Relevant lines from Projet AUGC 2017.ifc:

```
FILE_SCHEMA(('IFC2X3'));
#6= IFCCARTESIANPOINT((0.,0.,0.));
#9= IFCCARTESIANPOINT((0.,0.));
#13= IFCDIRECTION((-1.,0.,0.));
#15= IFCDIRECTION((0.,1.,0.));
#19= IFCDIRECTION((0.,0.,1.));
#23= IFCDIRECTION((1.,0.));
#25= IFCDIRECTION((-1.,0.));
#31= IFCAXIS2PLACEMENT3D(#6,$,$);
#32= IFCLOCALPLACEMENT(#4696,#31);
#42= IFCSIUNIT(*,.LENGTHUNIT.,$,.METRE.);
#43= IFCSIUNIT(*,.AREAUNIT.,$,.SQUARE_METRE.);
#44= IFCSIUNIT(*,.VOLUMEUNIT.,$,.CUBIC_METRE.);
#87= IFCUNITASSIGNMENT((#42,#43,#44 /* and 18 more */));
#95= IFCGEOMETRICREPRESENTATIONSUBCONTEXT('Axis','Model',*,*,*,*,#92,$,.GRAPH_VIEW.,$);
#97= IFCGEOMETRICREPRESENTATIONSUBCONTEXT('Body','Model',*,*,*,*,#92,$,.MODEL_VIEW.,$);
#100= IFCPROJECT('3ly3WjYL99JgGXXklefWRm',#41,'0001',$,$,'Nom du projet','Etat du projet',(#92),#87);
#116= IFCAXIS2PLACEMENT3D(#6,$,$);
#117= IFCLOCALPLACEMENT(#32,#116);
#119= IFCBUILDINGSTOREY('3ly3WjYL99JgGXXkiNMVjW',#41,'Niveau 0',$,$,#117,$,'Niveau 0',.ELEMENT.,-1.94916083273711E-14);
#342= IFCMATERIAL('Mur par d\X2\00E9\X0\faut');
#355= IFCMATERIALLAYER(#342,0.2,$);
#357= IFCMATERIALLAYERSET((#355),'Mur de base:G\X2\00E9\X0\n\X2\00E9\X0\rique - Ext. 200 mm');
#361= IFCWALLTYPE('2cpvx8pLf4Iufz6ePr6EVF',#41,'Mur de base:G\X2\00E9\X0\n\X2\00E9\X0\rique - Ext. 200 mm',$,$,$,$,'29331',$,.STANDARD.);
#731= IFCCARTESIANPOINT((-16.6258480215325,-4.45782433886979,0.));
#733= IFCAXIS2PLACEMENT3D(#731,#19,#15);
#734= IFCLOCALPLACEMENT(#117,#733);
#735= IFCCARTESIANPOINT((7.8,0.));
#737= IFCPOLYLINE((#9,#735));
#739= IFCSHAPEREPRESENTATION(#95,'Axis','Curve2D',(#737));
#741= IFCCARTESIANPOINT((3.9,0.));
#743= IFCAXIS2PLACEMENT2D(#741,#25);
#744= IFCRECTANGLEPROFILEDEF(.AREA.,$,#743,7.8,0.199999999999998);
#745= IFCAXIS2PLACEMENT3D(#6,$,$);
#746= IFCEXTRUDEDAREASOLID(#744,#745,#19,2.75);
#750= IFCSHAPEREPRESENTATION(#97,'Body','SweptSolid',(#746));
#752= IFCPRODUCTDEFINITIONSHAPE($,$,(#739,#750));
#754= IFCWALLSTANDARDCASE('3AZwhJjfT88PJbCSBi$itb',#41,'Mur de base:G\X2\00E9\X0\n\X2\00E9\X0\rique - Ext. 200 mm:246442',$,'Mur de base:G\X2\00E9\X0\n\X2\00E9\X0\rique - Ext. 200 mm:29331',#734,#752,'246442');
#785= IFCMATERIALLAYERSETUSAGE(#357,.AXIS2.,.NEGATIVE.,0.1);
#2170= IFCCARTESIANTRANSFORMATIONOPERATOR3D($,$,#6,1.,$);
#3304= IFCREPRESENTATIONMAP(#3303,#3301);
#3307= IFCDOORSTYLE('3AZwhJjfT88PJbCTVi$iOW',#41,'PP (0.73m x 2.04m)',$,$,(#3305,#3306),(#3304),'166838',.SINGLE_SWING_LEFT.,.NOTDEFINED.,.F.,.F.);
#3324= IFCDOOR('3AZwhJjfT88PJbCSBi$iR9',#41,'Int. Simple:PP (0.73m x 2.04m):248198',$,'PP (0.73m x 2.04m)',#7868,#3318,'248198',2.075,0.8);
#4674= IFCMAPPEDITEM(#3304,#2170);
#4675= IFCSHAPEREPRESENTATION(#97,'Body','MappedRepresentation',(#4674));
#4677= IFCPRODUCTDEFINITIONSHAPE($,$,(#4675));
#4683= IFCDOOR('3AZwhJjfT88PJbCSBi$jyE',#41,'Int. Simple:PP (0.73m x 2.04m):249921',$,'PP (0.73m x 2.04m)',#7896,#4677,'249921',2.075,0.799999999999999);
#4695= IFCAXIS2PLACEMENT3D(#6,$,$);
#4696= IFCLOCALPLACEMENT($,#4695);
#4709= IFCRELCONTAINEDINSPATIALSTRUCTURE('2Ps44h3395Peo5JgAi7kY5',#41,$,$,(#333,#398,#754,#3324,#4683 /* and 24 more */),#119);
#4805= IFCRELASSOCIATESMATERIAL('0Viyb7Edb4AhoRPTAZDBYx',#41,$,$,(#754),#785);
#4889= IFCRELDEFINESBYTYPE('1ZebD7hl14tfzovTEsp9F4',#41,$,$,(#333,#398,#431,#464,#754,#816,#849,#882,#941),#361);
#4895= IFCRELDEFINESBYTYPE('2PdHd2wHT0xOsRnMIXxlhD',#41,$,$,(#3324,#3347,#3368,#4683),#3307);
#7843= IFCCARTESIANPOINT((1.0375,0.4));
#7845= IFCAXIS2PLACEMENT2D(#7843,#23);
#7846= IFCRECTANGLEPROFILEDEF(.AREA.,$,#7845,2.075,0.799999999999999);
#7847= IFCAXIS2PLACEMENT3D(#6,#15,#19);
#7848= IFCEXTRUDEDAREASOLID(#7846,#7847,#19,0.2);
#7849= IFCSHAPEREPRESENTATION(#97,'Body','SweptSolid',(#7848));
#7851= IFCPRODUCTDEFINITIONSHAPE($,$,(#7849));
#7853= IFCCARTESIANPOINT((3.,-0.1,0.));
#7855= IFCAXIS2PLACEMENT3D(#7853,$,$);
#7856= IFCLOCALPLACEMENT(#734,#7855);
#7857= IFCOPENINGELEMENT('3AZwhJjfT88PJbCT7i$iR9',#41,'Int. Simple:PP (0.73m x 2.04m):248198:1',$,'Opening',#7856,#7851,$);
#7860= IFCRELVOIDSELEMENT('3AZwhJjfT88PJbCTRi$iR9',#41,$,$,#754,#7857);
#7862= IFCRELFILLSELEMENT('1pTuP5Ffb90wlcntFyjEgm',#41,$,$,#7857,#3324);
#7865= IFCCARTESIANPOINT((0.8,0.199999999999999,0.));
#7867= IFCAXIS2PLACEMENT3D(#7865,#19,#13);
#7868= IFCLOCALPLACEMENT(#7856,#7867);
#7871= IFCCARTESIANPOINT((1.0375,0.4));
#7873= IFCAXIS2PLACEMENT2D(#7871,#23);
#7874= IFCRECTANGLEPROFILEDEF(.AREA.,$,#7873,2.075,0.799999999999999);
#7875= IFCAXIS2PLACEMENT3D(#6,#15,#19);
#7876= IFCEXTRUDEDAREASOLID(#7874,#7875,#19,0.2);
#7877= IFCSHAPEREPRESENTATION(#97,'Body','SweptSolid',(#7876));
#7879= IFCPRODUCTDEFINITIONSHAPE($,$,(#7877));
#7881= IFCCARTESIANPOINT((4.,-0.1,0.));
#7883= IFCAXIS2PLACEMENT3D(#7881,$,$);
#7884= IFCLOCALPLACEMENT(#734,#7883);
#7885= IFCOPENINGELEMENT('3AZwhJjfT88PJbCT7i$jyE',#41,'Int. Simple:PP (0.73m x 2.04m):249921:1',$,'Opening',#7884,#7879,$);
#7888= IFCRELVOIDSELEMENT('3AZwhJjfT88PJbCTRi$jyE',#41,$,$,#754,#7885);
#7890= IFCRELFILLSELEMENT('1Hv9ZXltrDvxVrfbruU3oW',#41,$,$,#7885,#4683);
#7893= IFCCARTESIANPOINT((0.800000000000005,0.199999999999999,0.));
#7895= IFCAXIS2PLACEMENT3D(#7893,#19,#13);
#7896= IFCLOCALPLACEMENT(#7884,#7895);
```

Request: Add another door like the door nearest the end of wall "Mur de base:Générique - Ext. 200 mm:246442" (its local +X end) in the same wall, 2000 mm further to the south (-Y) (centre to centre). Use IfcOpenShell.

```python
import ifcopenshell
import ifcopenshell.api.feature
import ifcopenshell.api.geometry
import ifcopenshell.api.root
import ifcopenshell.geom
import ifcopenshell.util.element
import ifcopenshell.util.placement
import ifcopenshell.util.shape

model = ifcopenshell.open("Projet AUGC 2017.ifc")
settings = ifcopenshell.geom.settings()


def volume(element):
    """Net volume in cubic metres, openings subtracted."""
    shape = ifcopenshell.geom.create_shape(settings, element)
    return ifcopenshell.util.shape.get_volume(shape.geometry)


def reuse_history(source, copy):
    """copy_class also copies each property set's owner history, people and application; keep the originals."""
    for rel in copy.IsDefinedBy:
        if rel.is_a("IfcRelDefinesByProperties") and (history := rel.RelatingPropertyDefinition.OwnerHistory):
            rel.RelatingPropertyDefinition.OwnerHistory = source.OwnerHistory
            ifcopenshell.util.element.remove_deep2(model, history)


door = model.by_id(4683)
opening = door.FillsVoids[0].RelatingOpeningElement
wall = opening.VoidsElements[0].RelatingBuildingElement
before = volume(wall)
shift = ifcopenshell.util.placement.get_local_placement(wall.ObjectPlacement)[:3, 0] * -2.0

# copy_class copies the void relationship, type, container and properties, but no geometry.
new_opening = ifcopenshell.api.root.copy_class(model, product=opening)
new_opening.Representation = ifcopenshell.util.element.copy_deep(
    model, opening.Representation, exclude=["IfcGeometricRepresentationContext", "IfcRepresentationMap"]
)
new_opening.Name = "Int. Simple:PP (0.73m x 2.04m)"
new_door = ifcopenshell.api.root.copy_class(model, product=door)
new_door.Representation = ifcopenshell.util.element.copy_deep(
    model, door.Representation, exclude=["IfcGeometricRepresentationContext", "IfcRepresentationMap"]
)
new_door.Name = "Int. Simple:PP (0.73m x 2.04m)"
new_door.Tag = None
reuse_history(door, new_door)
fills = ifcopenshell.api.feature.add_filling(model, opening=new_opening, element=new_door)
fills.OwnerHistory = new_door.OwnerHistory  # required in IFC2X3

for old, new in ((opening, new_opening), (door, new_door)):
    matrix = ifcopenshell.util.placement.get_local_placement(old.ObjectPlacement)
    matrix[:3, 3] += shift
    ifcopenshell.api.geometry.edit_object_placement(model, product=new, matrix=matrix, is_si=False)

after = volume(wall)

print(f"wall volume {before:.3f} -> {after:.3f} m3")

model.write("Projet AUGC 2017_edited.ifc")
```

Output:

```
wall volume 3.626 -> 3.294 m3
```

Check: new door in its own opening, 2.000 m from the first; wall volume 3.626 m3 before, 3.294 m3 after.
